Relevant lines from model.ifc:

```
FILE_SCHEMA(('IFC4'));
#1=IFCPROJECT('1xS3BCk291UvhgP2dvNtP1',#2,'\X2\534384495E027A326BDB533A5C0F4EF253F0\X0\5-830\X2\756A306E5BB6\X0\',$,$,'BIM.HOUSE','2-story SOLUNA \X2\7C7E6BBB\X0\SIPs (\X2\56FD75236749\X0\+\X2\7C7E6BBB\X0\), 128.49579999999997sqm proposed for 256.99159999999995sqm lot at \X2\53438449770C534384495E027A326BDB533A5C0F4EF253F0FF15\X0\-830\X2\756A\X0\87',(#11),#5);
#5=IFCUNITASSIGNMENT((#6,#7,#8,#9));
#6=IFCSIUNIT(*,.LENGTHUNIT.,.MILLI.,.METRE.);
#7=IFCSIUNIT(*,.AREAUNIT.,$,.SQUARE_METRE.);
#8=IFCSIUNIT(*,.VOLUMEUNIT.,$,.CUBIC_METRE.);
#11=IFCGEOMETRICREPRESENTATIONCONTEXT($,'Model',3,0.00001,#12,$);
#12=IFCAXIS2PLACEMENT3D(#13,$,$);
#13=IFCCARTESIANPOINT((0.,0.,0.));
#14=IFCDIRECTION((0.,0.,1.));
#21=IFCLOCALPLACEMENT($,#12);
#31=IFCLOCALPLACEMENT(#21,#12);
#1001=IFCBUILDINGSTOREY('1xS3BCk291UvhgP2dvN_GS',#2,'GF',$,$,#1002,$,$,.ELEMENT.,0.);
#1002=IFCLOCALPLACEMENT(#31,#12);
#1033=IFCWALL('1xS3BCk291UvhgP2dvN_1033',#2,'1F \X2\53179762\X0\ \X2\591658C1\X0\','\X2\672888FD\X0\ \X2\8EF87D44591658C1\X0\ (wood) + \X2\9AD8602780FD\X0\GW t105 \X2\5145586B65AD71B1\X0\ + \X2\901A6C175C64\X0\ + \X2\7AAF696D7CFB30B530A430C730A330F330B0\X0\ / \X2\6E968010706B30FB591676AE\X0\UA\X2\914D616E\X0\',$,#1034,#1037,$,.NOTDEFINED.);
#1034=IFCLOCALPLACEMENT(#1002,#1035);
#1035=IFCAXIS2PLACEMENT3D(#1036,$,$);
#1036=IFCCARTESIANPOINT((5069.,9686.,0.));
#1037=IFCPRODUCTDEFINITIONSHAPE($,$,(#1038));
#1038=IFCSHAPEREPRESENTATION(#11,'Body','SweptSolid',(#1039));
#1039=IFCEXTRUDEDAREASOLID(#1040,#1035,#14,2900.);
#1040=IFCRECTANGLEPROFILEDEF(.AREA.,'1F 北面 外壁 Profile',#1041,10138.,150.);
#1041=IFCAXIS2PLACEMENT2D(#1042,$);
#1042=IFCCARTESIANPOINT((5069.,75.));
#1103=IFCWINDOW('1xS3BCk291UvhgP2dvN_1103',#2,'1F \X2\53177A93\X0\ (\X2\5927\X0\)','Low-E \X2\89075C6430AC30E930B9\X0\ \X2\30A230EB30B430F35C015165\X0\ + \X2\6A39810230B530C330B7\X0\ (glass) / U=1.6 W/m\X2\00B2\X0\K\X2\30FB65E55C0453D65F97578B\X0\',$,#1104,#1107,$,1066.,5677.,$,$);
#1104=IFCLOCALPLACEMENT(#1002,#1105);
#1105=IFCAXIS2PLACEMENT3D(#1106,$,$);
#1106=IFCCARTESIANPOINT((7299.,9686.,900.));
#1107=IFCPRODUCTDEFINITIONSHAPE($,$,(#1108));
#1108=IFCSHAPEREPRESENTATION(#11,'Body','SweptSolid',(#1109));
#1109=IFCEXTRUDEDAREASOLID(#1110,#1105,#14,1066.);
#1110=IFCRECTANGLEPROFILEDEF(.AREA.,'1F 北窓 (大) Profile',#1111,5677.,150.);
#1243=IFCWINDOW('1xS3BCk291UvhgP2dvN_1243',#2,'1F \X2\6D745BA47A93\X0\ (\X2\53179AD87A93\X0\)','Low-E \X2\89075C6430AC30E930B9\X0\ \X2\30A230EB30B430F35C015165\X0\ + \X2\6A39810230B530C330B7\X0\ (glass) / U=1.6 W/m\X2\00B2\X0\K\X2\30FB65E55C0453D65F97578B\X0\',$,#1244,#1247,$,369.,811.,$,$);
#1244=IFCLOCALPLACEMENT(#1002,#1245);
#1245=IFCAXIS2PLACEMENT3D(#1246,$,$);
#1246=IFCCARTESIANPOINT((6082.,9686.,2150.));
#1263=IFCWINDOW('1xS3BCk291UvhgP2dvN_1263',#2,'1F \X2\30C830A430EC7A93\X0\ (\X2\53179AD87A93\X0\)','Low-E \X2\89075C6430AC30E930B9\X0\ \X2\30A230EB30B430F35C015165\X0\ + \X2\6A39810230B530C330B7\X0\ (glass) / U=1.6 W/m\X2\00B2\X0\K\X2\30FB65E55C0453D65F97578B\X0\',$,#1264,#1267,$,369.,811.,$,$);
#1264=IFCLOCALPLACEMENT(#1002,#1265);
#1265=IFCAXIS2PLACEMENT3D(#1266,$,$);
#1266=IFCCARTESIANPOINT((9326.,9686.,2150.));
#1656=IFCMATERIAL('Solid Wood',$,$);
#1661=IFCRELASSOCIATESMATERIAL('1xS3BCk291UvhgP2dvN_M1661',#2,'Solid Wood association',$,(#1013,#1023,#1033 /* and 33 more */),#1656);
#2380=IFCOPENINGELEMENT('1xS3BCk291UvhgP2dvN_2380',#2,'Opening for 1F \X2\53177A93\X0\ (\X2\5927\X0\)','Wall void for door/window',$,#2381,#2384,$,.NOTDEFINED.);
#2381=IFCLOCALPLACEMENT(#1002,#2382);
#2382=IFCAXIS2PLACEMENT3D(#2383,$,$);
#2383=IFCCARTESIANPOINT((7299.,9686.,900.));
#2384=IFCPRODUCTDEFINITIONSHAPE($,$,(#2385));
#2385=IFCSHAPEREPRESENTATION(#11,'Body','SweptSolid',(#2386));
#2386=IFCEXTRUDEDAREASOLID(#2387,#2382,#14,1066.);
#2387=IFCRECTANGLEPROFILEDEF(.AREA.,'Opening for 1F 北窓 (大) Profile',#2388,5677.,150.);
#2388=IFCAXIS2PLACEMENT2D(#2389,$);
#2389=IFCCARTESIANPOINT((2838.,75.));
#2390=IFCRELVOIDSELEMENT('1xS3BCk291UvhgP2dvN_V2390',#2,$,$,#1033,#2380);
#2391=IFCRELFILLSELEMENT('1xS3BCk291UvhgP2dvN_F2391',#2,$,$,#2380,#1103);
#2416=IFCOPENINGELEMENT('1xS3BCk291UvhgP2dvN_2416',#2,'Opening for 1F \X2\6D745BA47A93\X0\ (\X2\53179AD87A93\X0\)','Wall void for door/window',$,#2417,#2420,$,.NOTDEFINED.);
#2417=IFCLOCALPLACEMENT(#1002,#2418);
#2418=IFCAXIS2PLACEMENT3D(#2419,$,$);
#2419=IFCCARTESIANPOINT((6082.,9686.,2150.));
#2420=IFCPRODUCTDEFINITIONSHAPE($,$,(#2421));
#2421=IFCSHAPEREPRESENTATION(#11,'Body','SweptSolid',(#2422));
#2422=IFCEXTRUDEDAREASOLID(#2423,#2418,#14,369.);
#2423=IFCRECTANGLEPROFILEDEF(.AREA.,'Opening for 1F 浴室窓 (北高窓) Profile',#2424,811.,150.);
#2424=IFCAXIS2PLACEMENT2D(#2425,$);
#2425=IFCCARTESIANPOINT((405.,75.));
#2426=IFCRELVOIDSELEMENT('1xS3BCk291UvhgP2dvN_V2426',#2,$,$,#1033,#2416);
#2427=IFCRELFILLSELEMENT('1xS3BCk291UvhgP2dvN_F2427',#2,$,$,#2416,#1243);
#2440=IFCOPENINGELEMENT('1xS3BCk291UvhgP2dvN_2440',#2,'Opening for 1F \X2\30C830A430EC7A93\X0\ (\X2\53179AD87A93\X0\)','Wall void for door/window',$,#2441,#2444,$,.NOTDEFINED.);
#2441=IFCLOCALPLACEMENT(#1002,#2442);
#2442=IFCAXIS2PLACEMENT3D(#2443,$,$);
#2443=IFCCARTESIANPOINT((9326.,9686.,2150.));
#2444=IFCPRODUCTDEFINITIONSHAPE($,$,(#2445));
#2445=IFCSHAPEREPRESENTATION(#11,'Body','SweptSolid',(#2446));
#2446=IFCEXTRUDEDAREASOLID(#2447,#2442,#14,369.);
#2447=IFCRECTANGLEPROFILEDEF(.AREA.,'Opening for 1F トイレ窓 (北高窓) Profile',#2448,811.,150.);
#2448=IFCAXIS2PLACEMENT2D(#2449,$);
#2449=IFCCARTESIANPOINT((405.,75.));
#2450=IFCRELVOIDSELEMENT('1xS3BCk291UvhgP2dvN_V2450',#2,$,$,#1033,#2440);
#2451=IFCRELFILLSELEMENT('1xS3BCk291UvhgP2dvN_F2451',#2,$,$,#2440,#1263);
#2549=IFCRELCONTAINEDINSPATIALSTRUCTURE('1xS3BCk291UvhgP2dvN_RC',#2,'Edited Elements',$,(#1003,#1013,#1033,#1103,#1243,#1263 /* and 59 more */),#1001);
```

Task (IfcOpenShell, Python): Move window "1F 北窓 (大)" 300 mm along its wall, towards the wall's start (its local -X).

```python
import ifcopenshell
import ifcopenshell.api.geometry
import ifcopenshell.util.placement
import ifcopenshell.util.unit

model = ifcopenshell.open("model.ifc")
unit_scale = ifcopenshell.util.unit.calculate_unit_scale(model)

window = model.by_guid("1xS3BCk291UvhgP2dvN_1103")
opening = window.FillsVoids[0].RelatingOpeningElement
wall = opening.VoidsElements[0].RelatingBuildingElement

wall_matrix = ifcopenshell.util.placement.get_local_placement(wall.ObjectPlacement)
shift = wall_matrix[:3, 0] * -0.3 / unit_scale
before = ifcopenshell.util.placement.get_local_placement(window.ObjectPlacement)[:3, 3].copy()

# The window is not placed relative to its opening, so move both.
for product in (opening, window):
    matrix = ifcopenshell.util.placement.get_local_placement(product.ObjectPlacement)
    matrix[:3, 3] += shift
    ifcopenshell.api.geometry.edit_object_placement(model, product=product, matrix=matrix, is_si=False)

after = ifcopenshell.util.placement.get_local_placement(window.ObjectPlacement)[:3, 3]
print("window moved by", (after - before).round(3) + 0.0)

model.write("model_edited.ifc")
```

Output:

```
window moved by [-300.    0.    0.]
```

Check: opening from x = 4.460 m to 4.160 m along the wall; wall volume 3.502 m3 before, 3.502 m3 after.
